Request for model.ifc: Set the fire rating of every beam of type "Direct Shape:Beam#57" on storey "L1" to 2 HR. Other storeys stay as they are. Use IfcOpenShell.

First a look at what the model holds.

```python
import ifcopenshell
import ifcopenshell.util.element

model = ifcopenshell.open("model.ifc")
print(model.schema)
storey = next(s for s in model.by_type("IfcBuildingStorey") if s.Name == "L1")
beams = [e for e in ifcopenshell.util.element.get_decomposition(storey) if e.is_a("IfcBeam")]
seen = {}
for e in beams:
    element_type = ifcopenshell.util.element.get_type(e)
    key = (element_type.Name if element_type != e and element_type else None, ifcopenshell.util.element.get_pset(e, "Pset_BeamCommon", "FireRating"))
    seen[key] = seen.get(key, 0) + 1
for (name, value), count in sorted(seen.items(), key=str):
    print(count, "x", name, "|", value)
```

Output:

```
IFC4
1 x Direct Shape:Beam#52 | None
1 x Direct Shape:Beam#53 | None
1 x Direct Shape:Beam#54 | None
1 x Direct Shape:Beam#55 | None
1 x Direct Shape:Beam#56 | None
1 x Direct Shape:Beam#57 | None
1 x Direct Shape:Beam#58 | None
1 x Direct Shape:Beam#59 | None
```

```python
import ifcopenshell
import ifcopenshell.api.pset
import ifcopenshell.util.element

model = ifcopenshell.open("model.ifc")

storey = next(s for s in model.by_type("IfcBuildingStorey") if s.Name == "L1")
beams = [e for e in ifcopenshell.util.element.get_decomposition(storey) if e.is_a("IfcBeam")]

count = 0
for e in beams:
    element_type = ifcopenshell.util.element.get_type(e)
    if element_type in (None, e) or element_type.Name != "Direct Shape:Beam#57":
        continue
    # add_pset returns the element's existing set when there is one.
    pset = ifcopenshell.api.pset.add_pset(model, product=e, name="Pset_BeamCommon")
    ifcopenshell.api.pset.edit_pset(model, pset=pset, properties={"FireRating": "2 HR"})
    count += 1

print(count, "beams updated")

model.write("model_v2.ifc")
```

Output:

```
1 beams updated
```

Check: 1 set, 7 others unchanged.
